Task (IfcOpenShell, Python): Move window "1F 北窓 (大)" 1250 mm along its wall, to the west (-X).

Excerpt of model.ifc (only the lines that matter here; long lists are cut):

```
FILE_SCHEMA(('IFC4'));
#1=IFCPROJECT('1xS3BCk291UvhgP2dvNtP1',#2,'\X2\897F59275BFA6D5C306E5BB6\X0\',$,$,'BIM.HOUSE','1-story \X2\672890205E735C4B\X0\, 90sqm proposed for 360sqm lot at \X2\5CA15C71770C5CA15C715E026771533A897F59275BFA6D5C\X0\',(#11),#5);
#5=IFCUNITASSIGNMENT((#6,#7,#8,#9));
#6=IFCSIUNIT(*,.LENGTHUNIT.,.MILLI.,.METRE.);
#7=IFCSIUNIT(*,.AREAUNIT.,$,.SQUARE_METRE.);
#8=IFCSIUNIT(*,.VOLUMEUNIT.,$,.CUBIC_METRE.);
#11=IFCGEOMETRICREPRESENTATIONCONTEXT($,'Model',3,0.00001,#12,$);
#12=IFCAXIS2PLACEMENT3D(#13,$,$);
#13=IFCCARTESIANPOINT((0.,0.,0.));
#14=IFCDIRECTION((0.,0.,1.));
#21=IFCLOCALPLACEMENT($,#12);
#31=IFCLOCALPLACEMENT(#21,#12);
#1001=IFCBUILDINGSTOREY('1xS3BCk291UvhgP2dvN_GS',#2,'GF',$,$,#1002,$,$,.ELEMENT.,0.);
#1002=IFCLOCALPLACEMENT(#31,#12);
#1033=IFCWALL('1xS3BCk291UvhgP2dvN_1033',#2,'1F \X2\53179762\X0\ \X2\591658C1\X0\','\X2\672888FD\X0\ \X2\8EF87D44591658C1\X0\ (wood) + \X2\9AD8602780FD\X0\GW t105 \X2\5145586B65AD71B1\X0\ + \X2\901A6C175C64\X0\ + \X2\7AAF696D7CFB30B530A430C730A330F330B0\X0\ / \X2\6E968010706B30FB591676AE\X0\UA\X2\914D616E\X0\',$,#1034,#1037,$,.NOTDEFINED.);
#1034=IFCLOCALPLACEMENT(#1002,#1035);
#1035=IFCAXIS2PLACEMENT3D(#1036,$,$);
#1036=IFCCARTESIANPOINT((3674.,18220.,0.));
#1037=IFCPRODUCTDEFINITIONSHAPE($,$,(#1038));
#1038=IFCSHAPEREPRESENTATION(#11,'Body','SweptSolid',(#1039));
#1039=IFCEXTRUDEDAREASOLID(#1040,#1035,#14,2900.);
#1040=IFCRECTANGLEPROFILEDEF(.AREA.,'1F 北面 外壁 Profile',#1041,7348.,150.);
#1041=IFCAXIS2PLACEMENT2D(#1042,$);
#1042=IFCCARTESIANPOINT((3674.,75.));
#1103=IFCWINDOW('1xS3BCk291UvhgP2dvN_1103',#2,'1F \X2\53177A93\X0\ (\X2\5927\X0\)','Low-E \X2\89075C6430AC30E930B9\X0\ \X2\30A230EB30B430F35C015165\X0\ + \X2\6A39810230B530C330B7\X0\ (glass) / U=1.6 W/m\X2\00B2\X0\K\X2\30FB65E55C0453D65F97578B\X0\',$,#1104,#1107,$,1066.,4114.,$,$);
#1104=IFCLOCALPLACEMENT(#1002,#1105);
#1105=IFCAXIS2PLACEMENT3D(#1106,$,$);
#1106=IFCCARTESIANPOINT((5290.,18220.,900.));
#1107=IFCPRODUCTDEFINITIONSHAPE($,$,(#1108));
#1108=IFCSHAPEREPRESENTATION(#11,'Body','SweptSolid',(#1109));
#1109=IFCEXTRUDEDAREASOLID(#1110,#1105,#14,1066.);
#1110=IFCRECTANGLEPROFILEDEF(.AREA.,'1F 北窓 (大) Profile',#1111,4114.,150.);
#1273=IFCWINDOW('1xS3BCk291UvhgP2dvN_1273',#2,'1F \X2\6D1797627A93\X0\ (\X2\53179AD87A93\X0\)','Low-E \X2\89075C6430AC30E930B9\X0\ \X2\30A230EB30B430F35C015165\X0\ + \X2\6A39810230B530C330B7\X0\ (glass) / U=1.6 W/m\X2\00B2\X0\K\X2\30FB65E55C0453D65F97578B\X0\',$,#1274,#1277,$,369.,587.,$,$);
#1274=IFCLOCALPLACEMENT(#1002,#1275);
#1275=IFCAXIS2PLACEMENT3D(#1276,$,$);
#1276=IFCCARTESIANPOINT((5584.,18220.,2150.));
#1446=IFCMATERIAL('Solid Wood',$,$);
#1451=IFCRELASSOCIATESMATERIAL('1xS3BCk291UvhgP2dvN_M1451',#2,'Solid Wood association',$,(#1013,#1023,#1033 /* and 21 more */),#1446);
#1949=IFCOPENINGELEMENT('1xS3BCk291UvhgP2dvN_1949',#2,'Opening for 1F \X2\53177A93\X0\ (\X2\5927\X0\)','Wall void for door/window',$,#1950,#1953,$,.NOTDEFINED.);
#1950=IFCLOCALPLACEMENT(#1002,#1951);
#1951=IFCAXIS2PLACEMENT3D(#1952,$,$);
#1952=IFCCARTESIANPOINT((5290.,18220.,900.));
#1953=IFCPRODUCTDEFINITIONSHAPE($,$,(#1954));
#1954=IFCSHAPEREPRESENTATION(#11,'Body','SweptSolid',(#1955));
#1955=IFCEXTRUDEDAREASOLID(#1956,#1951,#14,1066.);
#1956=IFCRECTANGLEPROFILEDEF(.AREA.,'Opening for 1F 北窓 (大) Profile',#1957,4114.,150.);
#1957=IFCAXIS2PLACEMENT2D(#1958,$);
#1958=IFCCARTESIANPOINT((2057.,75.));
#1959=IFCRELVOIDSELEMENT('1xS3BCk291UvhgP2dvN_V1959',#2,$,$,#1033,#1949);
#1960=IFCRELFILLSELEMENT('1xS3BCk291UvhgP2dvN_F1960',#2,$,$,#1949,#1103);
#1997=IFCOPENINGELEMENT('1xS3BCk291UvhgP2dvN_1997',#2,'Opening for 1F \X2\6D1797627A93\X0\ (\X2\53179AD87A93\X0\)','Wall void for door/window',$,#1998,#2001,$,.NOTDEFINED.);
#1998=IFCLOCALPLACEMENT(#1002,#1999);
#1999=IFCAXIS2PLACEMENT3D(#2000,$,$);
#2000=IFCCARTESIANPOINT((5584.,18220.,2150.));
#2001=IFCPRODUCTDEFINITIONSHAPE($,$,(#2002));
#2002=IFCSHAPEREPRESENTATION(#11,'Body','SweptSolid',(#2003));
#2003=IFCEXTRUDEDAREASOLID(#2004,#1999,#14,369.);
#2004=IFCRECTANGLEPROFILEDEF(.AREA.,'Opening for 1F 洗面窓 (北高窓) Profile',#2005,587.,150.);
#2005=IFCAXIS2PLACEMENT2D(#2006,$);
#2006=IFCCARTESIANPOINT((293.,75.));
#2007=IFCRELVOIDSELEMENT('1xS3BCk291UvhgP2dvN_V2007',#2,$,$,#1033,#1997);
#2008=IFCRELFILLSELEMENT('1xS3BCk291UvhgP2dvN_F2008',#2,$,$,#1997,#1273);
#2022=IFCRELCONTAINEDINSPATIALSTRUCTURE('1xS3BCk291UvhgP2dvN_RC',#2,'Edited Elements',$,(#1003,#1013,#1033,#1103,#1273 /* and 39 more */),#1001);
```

```python
import ifcopenshell
import ifcopenshell.api.geometry
import ifcopenshell.util.placement
import ifcopenshell.util.unit

model = ifcopenshell.open("model.ifc")
unit_scale = ifcopenshell.util.unit.calculate_unit_scale(model)

window = model.by_guid("1xS3BCk291UvhgP2dvN_1103")
opening = window.FillsVoids[0].RelatingOpeningElement
wall = opening.VoidsElements[0].RelatingBuildingElement

wall_matrix = ifcopenshell.util.placement.get_local_placement(wall.ObjectPlacement)
shift = wall_matrix[:3, 0] * -1.25 / unit_scale
before = ifcopenshell.util.placement.get_local_placement(window.ObjectPlacement)[:3, 3].copy()

# The window is not placed relative to its opening, so move both.
for product in (opening, window):
    matrix = ifcopenshell.util.placement.get_local_placement(product.ObjectPlacement)
    matrix[:3, 3] += shift
    ifcopenshell.api.geometry.edit_object_placement(model, product=product, matrix=matrix, is_si=False)

after = ifcopenshell.util.placement.get_local_placement(window.ObjectPlacement)[:3, 3]
print("window moved by", (after - before).round(3) + 0.0)

model.write("model-out.ifc")
```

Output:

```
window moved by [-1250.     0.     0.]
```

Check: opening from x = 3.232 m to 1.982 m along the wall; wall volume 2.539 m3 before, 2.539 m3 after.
